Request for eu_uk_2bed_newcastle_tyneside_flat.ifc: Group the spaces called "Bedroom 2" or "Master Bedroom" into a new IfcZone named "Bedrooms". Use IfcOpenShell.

First a look at what the model holds.

```python
import ifcopenshell

model = ifcopenshell.open("eu_uk_2bed_newcastle_tyneside_flat.ifc")
print(model.schema)
seen = {}
for space in model.by_type("IfcSpace"):
    seen[space.LongName] = seen.get(space.LongName, 0) + 1
for name, count in sorted(seen.items(), key=str):
    print(count, "x", name)
print("zones:", [z.Name for z in model.by_type("IfcZone")][:20])
```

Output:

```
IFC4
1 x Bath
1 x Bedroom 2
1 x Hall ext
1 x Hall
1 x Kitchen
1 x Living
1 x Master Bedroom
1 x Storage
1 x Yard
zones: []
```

```python
import ifcopenshell
import ifcopenshell.api.group
import ifcopenshell.api.root

model = ifcopenshell.open("eu_uk_2bed_newcastle_tyneside_flat.ifc")

names = {"Bedroom 2", "Master Bedroom"}
spaces = [s for s in model.by_type("IfcSpace") if s.LongName in names]

zone = ifcopenshell.api.root.create_entity(model, ifc_class="IfcZone", name="Bedrooms")
ifcopenshell.api.group.assign_group(model, products=spaces, group=zone)
print(len(spaces), "spaces in", zone.Name)

model.write("eu_uk_2bed_newcastle_tyneside_flat_rev.ifc")
```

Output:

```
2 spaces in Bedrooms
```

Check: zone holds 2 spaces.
